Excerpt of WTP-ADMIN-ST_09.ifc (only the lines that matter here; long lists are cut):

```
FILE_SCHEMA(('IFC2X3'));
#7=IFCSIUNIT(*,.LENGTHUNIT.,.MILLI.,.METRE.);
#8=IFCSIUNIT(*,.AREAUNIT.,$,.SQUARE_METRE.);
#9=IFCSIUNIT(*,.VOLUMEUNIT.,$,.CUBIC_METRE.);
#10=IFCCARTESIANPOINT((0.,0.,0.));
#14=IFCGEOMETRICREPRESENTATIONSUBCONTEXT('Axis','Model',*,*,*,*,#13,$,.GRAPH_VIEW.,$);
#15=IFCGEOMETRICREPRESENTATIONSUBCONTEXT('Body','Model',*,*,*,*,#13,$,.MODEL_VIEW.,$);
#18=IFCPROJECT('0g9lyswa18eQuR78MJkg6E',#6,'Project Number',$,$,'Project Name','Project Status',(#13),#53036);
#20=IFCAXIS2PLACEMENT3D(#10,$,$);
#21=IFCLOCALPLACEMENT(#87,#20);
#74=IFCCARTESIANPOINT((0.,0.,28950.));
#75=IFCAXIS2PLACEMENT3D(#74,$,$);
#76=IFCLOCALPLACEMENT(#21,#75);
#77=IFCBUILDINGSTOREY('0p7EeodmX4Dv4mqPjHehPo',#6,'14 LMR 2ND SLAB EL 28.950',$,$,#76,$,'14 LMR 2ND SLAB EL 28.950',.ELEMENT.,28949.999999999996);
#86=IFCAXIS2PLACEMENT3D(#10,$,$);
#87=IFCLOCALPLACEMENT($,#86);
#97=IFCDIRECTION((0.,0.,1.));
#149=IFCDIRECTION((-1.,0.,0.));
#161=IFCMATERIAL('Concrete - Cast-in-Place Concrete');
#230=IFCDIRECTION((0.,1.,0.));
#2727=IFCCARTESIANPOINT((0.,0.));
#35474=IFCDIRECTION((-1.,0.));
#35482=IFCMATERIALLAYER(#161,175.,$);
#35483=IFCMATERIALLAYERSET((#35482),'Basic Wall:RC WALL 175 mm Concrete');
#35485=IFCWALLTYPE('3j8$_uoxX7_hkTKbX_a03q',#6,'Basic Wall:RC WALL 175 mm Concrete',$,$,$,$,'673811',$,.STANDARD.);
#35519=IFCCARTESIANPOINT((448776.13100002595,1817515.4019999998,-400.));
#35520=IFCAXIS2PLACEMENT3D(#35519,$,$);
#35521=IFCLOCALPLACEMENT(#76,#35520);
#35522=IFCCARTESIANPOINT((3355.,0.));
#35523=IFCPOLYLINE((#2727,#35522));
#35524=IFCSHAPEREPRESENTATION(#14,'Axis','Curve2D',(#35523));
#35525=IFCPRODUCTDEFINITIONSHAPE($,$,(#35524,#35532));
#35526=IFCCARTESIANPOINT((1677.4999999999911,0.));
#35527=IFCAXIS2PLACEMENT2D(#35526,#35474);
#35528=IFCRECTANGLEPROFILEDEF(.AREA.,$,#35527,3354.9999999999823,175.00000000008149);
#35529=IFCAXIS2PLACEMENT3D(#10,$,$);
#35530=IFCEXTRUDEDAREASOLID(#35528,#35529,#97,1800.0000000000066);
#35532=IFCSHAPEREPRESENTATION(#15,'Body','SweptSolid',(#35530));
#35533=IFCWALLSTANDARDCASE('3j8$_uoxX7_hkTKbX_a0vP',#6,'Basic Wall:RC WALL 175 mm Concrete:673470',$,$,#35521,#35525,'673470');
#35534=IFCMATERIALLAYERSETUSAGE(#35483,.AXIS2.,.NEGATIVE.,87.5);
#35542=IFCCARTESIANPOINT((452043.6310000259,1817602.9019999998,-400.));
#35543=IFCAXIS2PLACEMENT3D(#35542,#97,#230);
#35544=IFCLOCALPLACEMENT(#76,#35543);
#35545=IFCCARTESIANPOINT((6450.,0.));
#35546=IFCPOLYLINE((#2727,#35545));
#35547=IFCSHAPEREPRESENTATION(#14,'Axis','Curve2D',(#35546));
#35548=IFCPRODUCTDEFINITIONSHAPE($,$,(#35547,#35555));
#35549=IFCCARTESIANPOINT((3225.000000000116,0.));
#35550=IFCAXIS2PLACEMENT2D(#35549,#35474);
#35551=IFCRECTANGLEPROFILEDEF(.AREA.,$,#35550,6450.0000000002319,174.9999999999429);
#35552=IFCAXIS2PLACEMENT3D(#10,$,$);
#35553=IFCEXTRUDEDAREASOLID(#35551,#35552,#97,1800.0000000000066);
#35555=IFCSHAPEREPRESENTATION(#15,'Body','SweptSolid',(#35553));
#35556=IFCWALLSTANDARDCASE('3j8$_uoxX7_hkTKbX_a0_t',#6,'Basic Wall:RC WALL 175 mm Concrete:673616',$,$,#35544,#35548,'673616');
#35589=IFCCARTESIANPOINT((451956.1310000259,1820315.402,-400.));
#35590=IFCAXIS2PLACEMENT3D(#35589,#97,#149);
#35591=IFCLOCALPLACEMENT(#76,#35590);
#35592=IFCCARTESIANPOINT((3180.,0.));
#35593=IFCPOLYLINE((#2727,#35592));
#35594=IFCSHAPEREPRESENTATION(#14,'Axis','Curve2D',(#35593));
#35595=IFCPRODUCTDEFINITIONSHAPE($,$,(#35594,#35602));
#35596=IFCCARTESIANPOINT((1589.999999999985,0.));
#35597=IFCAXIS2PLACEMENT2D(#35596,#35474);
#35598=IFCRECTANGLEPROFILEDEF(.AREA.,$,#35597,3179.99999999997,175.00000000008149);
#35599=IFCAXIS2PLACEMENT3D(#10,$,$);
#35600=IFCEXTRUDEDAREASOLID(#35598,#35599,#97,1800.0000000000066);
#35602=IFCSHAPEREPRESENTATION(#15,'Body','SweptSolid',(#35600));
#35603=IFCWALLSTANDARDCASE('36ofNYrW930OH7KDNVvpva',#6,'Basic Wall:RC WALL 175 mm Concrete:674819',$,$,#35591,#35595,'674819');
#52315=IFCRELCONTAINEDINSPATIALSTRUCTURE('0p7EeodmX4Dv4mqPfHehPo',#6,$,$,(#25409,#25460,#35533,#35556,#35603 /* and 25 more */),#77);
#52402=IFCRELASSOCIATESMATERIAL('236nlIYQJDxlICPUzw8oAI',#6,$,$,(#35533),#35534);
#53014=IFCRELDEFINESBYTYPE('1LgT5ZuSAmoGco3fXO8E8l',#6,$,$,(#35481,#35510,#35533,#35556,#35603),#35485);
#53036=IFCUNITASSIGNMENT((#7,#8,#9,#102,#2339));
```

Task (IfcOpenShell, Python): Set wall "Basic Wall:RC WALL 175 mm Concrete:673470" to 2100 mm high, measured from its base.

```python
import ifcopenshell
import ifcopenshell.geom
import ifcopenshell.util.representation
import ifcopenshell.util.shape
import ifcopenshell.util.unit

model = ifcopenshell.open("WTP-ADMIN-ST_09.ifc")
unit_scale = ifcopenshell.util.unit.calculate_unit_scale(model)
settings = ifcopenshell.geom.settings()


def volume(element):
    """Net volume in cubic metres, openings subtracted."""
    shape = ifcopenshell.geom.create_shape(settings, element)
    return ifcopenshell.util.shape.get_volume(shape.geometry)


wall = model.by_guid("3j8$_uoxX7_hkTKbX_a0vP")
before = volume(wall)

body = ifcopenshell.util.representation.get_representation(wall, "Model", "Body")
solid = body.Items[0]
old_height = solid.Depth
solid.Depth = 2.1 / unit_scale
after = volume(wall)

print(f"height {old_height:g} -> {solid.Depth:g}, volume {before:.3f} -> {after:.3f} m3")

model.write("WTP-ADMIN-ST_09_updated.ifc")
```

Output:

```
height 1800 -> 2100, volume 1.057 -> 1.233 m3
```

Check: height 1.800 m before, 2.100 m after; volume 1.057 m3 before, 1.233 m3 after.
